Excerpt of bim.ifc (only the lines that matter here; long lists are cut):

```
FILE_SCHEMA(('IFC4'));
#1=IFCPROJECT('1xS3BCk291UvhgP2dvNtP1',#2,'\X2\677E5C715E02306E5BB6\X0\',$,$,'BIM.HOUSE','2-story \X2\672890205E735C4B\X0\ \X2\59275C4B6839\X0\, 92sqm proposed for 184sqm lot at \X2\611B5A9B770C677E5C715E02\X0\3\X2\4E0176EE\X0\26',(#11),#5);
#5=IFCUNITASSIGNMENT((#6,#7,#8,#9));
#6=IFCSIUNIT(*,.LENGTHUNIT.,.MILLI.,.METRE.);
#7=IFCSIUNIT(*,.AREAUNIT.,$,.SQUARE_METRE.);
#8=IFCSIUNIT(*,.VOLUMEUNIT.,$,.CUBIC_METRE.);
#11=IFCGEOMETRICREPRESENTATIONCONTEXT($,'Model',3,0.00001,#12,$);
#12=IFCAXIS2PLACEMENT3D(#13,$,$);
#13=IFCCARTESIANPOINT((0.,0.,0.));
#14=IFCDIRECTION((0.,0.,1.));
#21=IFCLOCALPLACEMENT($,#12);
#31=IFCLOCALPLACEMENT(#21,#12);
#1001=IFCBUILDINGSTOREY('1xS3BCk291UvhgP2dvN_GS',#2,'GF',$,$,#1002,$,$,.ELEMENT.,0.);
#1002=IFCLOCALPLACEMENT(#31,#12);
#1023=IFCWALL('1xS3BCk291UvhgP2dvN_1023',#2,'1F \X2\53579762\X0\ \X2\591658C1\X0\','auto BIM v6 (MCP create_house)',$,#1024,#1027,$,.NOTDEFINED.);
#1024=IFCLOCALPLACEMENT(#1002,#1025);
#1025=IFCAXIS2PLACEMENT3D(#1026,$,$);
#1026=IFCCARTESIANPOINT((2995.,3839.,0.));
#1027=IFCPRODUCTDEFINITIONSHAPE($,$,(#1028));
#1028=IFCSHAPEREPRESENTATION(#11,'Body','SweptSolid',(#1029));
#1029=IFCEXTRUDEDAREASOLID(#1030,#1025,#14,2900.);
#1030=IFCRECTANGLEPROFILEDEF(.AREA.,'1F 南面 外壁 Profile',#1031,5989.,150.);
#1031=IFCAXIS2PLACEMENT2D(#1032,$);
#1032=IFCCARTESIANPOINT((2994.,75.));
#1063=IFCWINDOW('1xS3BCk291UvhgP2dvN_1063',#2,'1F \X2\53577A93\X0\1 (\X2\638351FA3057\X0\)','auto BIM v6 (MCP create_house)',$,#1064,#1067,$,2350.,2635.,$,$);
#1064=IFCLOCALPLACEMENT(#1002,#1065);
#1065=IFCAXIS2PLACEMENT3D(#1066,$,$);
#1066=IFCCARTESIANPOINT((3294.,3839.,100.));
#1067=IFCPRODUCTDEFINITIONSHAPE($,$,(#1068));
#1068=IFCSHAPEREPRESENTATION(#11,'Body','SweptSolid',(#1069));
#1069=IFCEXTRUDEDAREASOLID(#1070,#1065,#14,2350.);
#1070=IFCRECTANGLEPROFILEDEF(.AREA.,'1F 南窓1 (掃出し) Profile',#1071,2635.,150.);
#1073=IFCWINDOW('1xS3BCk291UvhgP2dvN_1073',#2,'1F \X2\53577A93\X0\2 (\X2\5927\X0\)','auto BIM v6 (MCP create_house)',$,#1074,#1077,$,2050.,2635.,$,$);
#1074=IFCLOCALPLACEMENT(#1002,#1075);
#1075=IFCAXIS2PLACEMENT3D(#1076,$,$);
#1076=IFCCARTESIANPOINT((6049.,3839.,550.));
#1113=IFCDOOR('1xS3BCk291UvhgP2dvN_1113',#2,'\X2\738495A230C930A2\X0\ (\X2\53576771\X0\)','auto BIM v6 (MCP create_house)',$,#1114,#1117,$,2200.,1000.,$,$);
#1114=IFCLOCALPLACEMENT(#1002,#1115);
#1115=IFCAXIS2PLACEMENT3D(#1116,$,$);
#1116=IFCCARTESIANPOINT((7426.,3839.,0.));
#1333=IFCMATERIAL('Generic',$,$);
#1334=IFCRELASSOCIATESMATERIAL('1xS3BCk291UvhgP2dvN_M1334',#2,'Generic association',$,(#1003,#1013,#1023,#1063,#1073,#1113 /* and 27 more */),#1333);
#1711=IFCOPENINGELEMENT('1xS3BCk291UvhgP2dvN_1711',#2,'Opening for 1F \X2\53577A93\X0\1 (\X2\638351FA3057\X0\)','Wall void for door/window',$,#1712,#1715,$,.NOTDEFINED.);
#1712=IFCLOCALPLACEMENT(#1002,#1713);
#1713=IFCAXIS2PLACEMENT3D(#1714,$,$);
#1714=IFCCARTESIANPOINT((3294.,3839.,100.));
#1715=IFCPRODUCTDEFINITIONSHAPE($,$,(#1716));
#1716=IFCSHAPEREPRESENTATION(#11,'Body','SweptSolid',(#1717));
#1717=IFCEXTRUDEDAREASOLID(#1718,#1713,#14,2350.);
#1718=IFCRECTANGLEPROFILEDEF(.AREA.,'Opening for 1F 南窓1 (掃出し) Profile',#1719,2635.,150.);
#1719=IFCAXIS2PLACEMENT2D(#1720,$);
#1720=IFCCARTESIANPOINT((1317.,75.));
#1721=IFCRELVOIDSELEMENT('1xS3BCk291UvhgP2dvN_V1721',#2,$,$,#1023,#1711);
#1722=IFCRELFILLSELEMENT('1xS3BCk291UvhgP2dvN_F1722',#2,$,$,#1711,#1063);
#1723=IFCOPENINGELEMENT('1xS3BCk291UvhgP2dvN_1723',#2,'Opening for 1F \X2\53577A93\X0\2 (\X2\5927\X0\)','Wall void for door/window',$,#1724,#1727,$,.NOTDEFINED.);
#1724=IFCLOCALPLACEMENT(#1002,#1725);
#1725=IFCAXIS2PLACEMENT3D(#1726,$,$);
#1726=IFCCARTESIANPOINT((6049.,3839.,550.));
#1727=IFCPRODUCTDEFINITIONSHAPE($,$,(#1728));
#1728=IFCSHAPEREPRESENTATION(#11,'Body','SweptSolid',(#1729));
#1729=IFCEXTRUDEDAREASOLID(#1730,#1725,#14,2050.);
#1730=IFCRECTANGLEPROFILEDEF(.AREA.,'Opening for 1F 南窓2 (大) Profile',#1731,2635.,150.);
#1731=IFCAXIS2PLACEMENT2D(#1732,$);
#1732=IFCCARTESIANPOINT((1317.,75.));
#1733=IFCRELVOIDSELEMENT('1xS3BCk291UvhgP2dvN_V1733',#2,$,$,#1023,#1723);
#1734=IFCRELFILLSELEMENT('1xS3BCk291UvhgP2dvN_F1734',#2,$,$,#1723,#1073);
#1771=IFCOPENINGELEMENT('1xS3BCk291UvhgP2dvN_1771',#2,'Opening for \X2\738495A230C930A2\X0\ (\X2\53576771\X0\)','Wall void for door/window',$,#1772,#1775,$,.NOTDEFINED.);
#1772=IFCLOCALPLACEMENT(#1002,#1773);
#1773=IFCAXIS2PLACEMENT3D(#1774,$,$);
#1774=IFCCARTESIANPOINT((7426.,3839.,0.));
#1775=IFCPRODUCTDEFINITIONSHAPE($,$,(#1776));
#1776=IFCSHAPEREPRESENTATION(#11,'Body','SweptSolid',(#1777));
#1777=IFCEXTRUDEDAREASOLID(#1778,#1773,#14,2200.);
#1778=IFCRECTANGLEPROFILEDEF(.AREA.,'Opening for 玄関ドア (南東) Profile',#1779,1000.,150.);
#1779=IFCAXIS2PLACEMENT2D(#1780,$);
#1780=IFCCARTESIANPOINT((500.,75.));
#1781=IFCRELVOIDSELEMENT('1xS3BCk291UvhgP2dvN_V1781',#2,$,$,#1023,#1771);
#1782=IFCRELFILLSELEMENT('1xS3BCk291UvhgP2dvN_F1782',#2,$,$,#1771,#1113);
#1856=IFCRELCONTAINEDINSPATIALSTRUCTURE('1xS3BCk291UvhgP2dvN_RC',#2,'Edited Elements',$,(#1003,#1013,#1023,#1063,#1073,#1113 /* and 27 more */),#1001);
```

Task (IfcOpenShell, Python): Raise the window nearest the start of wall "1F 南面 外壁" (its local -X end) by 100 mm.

```python
import numpy as np
import ifcopenshell
import ifcopenshell.api.geometry
import ifcopenshell.util.placement
import ifcopenshell.util.unit

model = ifcopenshell.open("bim.ifc")
unit_scale = ifcopenshell.util.unit.calculate_unit_scale(model)

window = model.by_guid("1xS3BCk291UvhgP2dvN_1063")
opening = window.FillsVoids[0].RelatingOpeningElement
dz = 0.1 / unit_scale

shift = np.array([0.0, 0.0, dz])
# The window is not placed relative to its opening, so move both.
for product in (opening, window):
    matrix = ifcopenshell.util.placement.get_local_placement(product.ObjectPlacement)
    matrix[:3, 3] += shift
    ifcopenshell.api.geometry.edit_object_placement(model, product=product, matrix=matrix, is_si=False)

print(f"moved by {dz * unit_scale:+.3f} m")

model.write("bim_updated.ifc")
```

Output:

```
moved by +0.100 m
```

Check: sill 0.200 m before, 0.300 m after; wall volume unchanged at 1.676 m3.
